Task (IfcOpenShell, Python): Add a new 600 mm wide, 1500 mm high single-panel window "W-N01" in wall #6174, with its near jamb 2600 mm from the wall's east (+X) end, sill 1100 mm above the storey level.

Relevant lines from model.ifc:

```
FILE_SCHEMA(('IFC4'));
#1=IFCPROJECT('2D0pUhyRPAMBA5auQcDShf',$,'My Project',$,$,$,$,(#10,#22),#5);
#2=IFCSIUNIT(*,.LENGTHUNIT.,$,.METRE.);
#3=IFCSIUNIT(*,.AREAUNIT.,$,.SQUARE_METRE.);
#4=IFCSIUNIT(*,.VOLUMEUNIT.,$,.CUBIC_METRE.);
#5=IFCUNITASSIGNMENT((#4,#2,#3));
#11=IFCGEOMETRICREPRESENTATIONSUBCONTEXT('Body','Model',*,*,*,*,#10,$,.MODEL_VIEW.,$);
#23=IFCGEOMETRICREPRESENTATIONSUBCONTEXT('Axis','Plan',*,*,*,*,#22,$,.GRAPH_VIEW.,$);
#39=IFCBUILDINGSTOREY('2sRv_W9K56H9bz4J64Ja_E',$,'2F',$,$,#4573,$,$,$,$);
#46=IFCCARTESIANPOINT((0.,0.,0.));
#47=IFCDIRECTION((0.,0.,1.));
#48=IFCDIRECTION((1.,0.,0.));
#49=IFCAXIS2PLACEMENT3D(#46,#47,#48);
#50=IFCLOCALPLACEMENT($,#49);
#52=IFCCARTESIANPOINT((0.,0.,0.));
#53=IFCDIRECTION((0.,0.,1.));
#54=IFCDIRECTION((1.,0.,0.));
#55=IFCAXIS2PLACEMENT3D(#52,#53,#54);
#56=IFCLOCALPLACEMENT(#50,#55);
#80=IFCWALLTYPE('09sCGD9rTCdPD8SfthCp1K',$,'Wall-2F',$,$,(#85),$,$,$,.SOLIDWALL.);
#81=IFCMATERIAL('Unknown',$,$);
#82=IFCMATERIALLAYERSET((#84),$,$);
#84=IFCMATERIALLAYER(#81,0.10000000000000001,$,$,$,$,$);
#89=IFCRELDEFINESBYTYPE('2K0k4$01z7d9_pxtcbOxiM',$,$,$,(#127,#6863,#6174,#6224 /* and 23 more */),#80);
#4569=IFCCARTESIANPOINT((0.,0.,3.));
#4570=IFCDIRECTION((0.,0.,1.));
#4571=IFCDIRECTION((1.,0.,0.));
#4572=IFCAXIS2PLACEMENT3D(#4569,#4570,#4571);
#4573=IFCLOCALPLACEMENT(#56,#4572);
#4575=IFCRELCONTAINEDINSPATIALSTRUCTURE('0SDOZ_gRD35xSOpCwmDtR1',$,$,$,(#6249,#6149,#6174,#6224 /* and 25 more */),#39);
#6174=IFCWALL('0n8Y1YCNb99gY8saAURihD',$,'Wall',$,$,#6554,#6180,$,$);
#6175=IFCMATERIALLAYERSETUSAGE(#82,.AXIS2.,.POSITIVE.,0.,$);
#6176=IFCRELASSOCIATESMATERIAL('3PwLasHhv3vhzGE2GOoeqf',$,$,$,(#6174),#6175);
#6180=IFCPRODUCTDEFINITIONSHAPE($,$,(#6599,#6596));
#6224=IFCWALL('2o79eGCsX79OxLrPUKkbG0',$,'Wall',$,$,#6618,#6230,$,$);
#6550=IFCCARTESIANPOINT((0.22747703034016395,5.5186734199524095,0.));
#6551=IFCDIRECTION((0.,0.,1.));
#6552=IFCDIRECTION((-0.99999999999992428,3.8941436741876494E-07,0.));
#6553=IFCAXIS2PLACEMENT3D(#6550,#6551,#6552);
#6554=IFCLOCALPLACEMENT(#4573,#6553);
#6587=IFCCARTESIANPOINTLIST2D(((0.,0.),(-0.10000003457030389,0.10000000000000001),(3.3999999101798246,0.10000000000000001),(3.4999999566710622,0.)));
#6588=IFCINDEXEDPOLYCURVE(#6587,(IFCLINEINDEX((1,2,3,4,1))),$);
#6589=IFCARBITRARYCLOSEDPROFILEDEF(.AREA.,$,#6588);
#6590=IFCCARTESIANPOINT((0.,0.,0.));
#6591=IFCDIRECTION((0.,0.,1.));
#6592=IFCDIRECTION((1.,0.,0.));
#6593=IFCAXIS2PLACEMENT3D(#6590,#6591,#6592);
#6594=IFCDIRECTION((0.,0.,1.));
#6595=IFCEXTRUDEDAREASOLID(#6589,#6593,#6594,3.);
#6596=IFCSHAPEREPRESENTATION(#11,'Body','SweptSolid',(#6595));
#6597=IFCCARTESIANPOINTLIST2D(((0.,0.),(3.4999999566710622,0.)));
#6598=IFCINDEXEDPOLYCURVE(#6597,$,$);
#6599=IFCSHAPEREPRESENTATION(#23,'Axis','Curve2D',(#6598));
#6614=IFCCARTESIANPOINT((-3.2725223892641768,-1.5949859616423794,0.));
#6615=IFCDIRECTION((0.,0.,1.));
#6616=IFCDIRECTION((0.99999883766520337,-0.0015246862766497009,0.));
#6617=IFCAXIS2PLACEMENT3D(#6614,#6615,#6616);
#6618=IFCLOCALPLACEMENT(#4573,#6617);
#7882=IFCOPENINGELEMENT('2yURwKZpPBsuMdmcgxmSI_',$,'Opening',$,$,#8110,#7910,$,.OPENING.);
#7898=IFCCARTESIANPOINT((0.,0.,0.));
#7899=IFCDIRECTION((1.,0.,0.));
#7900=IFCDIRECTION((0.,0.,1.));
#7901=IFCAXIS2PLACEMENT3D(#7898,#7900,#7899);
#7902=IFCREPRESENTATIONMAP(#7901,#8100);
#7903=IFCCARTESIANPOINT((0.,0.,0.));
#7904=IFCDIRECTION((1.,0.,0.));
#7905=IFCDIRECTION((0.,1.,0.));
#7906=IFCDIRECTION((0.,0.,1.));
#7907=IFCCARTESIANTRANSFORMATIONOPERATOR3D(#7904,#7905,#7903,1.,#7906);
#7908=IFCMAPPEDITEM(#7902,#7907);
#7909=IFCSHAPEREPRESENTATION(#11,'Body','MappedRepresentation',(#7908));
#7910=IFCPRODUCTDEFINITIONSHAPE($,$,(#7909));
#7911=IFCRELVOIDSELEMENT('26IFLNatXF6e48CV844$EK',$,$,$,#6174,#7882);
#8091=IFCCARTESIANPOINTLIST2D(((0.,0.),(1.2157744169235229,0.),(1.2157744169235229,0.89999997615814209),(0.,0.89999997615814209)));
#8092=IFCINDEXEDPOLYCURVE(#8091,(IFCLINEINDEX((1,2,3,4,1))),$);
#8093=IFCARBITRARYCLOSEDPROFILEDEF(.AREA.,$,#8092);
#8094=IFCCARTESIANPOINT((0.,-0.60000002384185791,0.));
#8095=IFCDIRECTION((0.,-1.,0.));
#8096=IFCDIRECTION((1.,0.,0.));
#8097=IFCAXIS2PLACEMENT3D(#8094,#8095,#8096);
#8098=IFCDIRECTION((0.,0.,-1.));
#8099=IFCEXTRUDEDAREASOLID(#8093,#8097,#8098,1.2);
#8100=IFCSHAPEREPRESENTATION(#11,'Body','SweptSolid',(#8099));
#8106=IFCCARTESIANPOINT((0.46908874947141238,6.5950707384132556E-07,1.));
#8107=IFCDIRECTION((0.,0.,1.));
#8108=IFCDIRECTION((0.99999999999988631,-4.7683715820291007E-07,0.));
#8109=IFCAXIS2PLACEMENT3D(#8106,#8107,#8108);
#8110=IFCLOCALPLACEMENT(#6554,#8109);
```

```python
import numpy as np
import ifcopenshell
import ifcopenshell.api.feature
import ifcopenshell.api.geometry
import ifcopenshell.api.root
import ifcopenshell.api.spatial
import ifcopenshell.geom
import ifcopenshell.util.element
import ifcopenshell.util.placement
import ifcopenshell.util.representation
import ifcopenshell.util.shape
import ifcopenshell.util.unit

model = ifcopenshell.open("model.ifc")
unit_scale = ifcopenshell.util.unit.calculate_unit_scale(model)
settings = ifcopenshell.geom.settings()


def volume(element):
    """Net volume in cubic metres, openings subtracted."""
    shape = ifcopenshell.geom.create_shape(settings, element)
    return ifcopenshell.util.shape.get_volume(shape.geometry)


wall = model.by_guid("0n8Y1YCNb99gY8saAURihD")
storey = ifcopenshell.util.element.get_container(wall, ifc_class="IfcBuildingStorey")
context = ifcopenshell.util.representation.get_context(model, "Model", "Body", "MODEL_VIEW")
before = volume(wall)

width, height, from_end, sill = 0.6, 1.5, 2.6, 1.1  # metres

# The wall runs along its own X axis, and the end named is its -X end.
wall_shape = ifcopenshell.geom.create_shape(settings, wall)
x, y, z = ifcopenshell.util.shape.get_vertices(wall_shape.geometry).T
start = x.min() + from_end
face, thickness = float(y.min()), float(y.max() - y.min())
wall_matrix = ifcopenshell.util.placement.get_local_placement(wall.ObjectPlacement)
level = ifcopenshell.util.placement.get_local_placement(storey.ObjectPlacement)[2, 3]


def in_wall(x, y):
    """Placement at x, y metres in the wall's axes, at sill height."""
    matrix = wall_matrix.copy()
    matrix[:, 3] = wall_matrix @ np.array([x / unit_scale, y / unit_scale, 0.0, 1.0])
    matrix[2, 3] = level + sill / unit_scale
    return matrix


# Opening: a box that overshoots both wall faces by 50 mm.
opening = ifcopenshell.api.root.create_entity(model, ifc_class="IfcOpeningElement", predefined_type="OPENING")
box = ifcopenshell.api.geometry.add_wall_representation(
    model, context=context, length=width, height=height, thickness=thickness + 0.1
)
ifcopenshell.api.geometry.assign_representation(model, product=opening, representation=box)
ifcopenshell.api.geometry.edit_object_placement(model, product=opening, matrix=in_wall(start, face - 0.05), is_si=False)
ifcopenshell.api.feature.add_feature(model, feature=opening, element=wall)

window = ifcopenshell.api.root.create_entity(model, ifc_class="IfcWindow", name="W-N01", predefined_type="WINDOW")
window.OverallWidth, window.OverallHeight = width / unit_scale, height / unit_scale
window.PartitioningType = "SINGLE_PANEL"
body = ifcopenshell.api.geometry.add_window_representation(
    model,
    context=context,
    overall_width=window.OverallWidth,
    overall_height=window.OverallHeight,
    partition_type="SINGLE_PANEL",
)
ifcopenshell.api.geometry.assign_representation(model, product=window, representation=body)
ifcopenshell.api.spatial.assign_container(model, products=[window], relating_structure=storey)
ifcopenshell.api.feature.add_filling(model, opening=opening, element=window)

# Centre the window in the wall's thickness.
ifcopenshell.api.geometry.edit_object_placement(model, product=window, matrix=in_wall(start, face), is_si=False)
window_shape = ifcopenshell.geom.create_shape(settings, window)
depth = ifcopenshell.util.shape.get_vertices(window_shape.geometry)[:, 1]
offset = face + thickness / 2 - (depth.min() + depth.max()) / 2
ifcopenshell.api.geometry.edit_object_placement(model, product=window, matrix=in_wall(start, offset), is_si=False)

after = volume(wall)

print(f"wall volume {before:.3f} -> {after:.3f} m3")

model.write("model_edited.ifc")
```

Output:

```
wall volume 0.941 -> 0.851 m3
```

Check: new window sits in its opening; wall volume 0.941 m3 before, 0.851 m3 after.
